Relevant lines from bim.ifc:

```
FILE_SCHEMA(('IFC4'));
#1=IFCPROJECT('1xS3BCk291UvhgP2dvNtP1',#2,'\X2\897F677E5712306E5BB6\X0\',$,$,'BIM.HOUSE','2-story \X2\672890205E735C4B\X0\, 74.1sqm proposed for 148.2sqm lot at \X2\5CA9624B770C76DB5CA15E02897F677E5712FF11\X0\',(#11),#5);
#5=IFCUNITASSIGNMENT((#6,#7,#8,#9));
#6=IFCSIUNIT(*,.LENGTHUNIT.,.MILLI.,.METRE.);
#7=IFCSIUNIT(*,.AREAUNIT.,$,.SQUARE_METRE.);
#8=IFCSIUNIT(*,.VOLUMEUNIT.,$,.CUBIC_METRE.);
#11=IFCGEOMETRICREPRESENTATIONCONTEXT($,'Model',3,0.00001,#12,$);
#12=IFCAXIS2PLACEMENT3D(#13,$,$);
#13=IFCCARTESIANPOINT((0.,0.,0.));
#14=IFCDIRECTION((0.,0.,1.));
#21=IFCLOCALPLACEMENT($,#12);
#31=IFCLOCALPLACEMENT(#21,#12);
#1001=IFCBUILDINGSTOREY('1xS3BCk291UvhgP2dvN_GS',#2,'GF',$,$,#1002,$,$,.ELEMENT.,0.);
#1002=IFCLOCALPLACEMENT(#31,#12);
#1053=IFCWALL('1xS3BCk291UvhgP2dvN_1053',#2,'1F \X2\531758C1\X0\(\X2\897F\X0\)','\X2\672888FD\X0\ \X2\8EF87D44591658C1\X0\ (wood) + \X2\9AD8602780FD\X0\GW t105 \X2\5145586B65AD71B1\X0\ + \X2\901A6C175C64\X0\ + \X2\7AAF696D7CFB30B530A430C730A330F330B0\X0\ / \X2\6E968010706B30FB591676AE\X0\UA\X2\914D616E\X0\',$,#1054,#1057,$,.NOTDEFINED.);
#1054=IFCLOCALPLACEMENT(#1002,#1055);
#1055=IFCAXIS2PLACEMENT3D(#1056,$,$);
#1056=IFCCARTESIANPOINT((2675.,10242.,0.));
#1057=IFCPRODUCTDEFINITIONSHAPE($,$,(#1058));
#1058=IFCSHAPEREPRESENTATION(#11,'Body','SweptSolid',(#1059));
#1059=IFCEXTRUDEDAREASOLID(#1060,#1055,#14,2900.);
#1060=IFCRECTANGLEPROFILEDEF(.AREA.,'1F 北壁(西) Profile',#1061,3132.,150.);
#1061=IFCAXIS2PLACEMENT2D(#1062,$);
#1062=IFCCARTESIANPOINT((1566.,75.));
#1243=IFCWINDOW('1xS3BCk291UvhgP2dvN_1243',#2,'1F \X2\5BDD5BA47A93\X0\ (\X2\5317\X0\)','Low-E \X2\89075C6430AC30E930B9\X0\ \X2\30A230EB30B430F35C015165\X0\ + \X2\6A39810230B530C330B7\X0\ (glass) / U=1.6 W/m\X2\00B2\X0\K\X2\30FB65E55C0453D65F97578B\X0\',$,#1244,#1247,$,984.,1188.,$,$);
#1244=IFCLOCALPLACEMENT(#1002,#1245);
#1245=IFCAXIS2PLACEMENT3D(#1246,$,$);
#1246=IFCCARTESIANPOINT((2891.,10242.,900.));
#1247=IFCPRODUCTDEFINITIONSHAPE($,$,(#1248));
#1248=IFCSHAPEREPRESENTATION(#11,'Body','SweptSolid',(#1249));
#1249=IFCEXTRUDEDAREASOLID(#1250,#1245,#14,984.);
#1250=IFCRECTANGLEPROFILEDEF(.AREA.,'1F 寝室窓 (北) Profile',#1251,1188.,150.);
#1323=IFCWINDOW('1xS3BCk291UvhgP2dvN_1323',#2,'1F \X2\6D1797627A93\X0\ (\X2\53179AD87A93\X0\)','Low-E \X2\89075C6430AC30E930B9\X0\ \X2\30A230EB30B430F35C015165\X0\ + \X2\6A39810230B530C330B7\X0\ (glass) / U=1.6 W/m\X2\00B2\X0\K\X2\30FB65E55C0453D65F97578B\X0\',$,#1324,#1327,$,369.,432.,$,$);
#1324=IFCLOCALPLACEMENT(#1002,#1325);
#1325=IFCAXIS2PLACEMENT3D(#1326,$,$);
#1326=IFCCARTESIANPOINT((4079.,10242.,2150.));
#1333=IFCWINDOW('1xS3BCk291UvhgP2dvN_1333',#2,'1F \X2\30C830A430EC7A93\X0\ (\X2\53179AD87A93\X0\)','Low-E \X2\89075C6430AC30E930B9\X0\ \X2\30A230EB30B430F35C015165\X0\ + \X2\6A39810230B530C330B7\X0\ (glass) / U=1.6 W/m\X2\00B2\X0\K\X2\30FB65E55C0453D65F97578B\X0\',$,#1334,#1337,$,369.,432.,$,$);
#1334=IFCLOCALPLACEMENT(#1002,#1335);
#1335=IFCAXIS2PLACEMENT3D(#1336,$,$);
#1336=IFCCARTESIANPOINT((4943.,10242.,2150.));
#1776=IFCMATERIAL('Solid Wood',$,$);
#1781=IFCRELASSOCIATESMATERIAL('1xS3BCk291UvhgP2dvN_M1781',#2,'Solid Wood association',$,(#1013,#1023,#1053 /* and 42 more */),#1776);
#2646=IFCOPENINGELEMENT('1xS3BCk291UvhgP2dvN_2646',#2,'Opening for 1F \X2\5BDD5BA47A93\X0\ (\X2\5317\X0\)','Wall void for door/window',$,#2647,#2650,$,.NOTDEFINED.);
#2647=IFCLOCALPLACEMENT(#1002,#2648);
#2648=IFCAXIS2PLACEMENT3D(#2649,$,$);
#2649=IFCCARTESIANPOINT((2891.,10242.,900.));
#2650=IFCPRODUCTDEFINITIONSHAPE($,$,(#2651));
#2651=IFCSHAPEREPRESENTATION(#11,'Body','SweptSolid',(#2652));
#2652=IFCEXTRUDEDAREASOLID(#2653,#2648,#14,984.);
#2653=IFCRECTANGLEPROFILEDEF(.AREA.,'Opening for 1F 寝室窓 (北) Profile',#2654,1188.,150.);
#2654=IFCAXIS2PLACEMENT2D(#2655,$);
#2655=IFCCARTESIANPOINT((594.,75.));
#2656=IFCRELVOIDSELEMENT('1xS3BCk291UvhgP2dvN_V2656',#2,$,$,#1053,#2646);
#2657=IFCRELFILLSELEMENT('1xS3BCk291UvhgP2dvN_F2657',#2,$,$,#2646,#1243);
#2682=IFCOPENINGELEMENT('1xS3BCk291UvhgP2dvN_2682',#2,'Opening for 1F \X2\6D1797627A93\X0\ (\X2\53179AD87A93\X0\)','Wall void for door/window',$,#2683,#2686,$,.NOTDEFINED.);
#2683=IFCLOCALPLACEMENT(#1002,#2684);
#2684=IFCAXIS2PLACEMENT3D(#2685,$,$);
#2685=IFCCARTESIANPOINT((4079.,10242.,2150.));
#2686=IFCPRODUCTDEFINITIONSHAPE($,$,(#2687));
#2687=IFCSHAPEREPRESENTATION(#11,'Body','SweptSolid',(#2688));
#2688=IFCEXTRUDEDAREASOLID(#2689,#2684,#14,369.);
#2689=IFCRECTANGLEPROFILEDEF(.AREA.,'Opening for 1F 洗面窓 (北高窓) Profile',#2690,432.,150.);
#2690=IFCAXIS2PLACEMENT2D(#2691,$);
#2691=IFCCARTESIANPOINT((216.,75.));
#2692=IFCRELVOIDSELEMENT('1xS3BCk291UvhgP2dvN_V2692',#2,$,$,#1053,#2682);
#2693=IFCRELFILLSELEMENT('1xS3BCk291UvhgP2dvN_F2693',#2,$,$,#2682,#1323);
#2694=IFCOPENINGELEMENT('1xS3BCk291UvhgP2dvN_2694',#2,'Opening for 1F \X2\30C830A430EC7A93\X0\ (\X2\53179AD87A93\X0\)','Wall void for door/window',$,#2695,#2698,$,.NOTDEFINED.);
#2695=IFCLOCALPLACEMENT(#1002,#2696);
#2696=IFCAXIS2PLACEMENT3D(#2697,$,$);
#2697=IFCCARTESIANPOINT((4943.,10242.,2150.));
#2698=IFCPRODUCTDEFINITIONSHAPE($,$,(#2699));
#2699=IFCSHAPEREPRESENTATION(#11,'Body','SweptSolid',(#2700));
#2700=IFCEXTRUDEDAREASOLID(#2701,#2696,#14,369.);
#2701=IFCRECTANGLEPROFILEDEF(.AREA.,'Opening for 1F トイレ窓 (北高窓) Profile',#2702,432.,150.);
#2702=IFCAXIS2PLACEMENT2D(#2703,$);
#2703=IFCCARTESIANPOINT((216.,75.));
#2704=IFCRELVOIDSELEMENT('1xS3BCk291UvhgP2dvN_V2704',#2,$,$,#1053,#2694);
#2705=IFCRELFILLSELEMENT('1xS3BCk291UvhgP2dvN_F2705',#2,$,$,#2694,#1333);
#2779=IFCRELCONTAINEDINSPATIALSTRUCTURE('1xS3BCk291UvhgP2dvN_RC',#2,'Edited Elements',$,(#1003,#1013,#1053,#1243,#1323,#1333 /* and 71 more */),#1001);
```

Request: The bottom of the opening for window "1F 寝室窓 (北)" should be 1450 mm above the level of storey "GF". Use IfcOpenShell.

```python
import numpy as np
import ifcopenshell
import ifcopenshell.api.geometry
import ifcopenshell.geom
import ifcopenshell.util.element
import ifcopenshell.util.placement
import ifcopenshell.util.shape
import ifcopenshell.util.unit

model = ifcopenshell.open("bim.ifc")
unit_scale = ifcopenshell.util.unit.calculate_unit_scale(model)

window = model.by_guid("1xS3BCk291UvhgP2dvN_1243")
opening = window.FillsVoids[0].RelatingOpeningElement
storey = ifcopenshell.util.element.get_container(window, ifc_class="IfcBuildingStorey")
level = ifcopenshell.util.placement.get_local_placement(storey.ObjectPlacement)[2, 3]

# The opening's origin need not be at the sill, so measure its lowest point.
shape = ifcopenshell.geom.create_shape(ifcopenshell.geom.settings(), opening)
bottom = ifcopenshell.util.shape.get_shape_bottom_elevation(shape, shape.geometry) / unit_scale
dz = level + 1450.0 - bottom

shift = np.array([0.0, 0.0, dz])
# The window is not placed relative to its opening, so move both.
for product in (opening, window):
    matrix = ifcopenshell.util.placement.get_local_placement(product.ObjectPlacement)
    matrix[:3, 3] += shift
    ifcopenshell.api.geometry.edit_object_placement(model, product=product, matrix=matrix, is_si=False)

print(f"moved by {dz * unit_scale:+.3f} m")

model.write("bim-out.ifc")
```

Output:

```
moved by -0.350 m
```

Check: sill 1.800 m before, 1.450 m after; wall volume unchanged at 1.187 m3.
